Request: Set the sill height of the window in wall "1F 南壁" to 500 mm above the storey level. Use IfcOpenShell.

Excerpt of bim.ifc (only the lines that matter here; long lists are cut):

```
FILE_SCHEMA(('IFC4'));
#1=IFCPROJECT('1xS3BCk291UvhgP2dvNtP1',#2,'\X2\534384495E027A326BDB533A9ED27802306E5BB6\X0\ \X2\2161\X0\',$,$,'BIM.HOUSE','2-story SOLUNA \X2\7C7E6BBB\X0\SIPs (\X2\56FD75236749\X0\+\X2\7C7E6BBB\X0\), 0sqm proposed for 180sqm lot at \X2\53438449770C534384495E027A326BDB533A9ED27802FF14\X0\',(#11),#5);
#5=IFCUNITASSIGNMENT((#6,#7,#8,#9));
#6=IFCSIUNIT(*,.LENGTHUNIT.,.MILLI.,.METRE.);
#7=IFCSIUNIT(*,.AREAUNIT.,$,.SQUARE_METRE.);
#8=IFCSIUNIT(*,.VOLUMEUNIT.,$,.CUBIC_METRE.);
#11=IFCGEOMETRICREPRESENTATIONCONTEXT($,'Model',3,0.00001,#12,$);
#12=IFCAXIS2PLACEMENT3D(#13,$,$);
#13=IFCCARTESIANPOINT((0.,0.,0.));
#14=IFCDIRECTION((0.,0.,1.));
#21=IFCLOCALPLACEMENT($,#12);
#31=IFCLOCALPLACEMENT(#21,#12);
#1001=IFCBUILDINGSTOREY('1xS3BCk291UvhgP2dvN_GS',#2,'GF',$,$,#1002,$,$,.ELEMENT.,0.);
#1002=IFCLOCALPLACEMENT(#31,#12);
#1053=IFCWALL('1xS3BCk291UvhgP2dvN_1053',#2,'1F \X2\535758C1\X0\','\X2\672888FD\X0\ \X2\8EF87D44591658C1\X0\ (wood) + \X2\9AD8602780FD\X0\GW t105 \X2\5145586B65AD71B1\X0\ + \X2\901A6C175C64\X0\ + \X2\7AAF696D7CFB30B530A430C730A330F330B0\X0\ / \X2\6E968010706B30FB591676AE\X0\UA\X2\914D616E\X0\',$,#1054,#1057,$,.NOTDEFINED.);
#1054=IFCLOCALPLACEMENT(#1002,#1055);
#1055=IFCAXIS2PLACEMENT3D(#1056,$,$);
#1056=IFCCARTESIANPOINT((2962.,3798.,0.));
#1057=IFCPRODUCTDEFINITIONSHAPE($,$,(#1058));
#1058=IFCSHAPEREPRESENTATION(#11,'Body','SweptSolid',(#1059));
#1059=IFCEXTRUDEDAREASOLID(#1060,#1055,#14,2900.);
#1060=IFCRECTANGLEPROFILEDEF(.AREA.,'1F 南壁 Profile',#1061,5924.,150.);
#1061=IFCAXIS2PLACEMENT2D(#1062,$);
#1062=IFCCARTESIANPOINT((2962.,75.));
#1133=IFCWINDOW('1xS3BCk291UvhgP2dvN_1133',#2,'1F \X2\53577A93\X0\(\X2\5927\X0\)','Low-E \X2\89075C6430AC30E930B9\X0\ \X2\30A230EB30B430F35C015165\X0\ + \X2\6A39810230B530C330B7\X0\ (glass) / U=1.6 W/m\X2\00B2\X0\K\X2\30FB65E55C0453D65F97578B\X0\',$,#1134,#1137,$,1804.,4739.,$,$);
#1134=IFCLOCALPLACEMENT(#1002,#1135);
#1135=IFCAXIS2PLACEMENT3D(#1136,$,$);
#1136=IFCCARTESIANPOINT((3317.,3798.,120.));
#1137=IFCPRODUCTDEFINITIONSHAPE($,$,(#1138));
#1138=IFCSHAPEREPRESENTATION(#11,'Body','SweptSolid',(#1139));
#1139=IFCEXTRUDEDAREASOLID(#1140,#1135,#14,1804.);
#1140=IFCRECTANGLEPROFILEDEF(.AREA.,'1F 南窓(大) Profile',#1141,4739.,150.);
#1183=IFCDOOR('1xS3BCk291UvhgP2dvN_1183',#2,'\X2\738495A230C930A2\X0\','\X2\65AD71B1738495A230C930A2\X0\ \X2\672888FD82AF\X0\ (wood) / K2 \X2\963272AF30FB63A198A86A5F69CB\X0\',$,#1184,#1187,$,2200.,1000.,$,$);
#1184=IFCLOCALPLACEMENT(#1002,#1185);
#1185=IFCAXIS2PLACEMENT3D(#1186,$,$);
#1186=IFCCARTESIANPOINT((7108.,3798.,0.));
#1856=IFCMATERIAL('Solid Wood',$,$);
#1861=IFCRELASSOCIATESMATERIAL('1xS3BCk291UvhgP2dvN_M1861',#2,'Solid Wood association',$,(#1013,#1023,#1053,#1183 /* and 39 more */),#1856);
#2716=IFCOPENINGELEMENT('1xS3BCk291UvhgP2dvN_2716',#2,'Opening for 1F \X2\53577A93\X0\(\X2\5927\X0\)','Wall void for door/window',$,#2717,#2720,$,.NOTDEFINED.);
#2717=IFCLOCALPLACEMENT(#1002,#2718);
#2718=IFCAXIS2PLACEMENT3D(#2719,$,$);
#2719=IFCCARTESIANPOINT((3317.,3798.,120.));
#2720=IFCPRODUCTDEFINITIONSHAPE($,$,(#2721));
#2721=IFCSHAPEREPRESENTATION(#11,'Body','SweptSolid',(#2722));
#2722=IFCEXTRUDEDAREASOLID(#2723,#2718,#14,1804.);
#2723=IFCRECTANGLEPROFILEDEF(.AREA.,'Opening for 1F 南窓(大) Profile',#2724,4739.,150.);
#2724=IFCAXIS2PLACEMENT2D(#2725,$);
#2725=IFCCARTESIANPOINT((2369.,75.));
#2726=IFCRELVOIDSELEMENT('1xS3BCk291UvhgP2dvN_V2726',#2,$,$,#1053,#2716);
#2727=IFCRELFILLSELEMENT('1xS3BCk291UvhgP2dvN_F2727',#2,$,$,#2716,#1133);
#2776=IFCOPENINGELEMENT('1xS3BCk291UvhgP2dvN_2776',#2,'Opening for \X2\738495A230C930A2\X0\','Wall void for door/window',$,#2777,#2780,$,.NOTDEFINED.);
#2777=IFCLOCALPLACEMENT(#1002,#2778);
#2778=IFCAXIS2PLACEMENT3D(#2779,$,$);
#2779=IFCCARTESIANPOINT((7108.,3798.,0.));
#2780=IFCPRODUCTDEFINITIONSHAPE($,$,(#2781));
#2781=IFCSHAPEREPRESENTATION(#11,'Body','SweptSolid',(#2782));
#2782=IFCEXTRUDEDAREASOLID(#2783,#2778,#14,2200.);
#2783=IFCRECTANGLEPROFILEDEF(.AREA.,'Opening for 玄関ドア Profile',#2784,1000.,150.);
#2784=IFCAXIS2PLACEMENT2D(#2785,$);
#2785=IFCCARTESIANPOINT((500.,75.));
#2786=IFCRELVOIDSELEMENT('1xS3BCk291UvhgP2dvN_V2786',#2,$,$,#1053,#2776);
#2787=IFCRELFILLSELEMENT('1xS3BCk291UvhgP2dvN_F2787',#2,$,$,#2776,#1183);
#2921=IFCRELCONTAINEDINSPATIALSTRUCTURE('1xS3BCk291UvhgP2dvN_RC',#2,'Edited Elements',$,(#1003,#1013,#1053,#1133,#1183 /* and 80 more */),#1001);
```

```python
import numpy as np
import ifcopenshell
import ifcopenshell.api.geometry
import ifcopenshell.geom
import ifcopenshell.util.element
import ifcopenshell.util.placement
import ifcopenshell.util.shape
import ifcopenshell.util.unit

model = ifcopenshell.open("bim.ifc")
unit_scale = ifcopenshell.util.unit.calculate_unit_scale(model)

window = model.by_guid("1xS3BCk291UvhgP2dvN_1133")
opening = window.FillsVoids[0].RelatingOpeningElement
storey = ifcopenshell.util.element.get_container(window, ifc_class="IfcBuildingStorey")
level = ifcopenshell.util.placement.get_local_placement(storey.ObjectPlacement)[2, 3]

# The opening's origin need not be at the sill, so measure its lowest point.
shape = ifcopenshell.geom.create_shape(ifcopenshell.geom.settings(), opening)
bottom = ifcopenshell.util.shape.get_shape_bottom_elevation(shape, shape.geometry) / unit_scale
dz = level + 500.0 - bottom

shift = np.array([0.0, 0.0, dz])
# The window is not placed relative to its opening, so move both.
for product in (opening, window):
    matrix = ifcopenshell.util.placement.get_local_placement(product.ObjectPlacement)
    matrix[:3, 3] += shift
    ifcopenshell.api.geometry.edit_object_placement(model, product=product, matrix=matrix, is_si=False)

print(f"moved by {dz * unit_scale:+.3f} m")

model.write("bim_edited.ifc")
```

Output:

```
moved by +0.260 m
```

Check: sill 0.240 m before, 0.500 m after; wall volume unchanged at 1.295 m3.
